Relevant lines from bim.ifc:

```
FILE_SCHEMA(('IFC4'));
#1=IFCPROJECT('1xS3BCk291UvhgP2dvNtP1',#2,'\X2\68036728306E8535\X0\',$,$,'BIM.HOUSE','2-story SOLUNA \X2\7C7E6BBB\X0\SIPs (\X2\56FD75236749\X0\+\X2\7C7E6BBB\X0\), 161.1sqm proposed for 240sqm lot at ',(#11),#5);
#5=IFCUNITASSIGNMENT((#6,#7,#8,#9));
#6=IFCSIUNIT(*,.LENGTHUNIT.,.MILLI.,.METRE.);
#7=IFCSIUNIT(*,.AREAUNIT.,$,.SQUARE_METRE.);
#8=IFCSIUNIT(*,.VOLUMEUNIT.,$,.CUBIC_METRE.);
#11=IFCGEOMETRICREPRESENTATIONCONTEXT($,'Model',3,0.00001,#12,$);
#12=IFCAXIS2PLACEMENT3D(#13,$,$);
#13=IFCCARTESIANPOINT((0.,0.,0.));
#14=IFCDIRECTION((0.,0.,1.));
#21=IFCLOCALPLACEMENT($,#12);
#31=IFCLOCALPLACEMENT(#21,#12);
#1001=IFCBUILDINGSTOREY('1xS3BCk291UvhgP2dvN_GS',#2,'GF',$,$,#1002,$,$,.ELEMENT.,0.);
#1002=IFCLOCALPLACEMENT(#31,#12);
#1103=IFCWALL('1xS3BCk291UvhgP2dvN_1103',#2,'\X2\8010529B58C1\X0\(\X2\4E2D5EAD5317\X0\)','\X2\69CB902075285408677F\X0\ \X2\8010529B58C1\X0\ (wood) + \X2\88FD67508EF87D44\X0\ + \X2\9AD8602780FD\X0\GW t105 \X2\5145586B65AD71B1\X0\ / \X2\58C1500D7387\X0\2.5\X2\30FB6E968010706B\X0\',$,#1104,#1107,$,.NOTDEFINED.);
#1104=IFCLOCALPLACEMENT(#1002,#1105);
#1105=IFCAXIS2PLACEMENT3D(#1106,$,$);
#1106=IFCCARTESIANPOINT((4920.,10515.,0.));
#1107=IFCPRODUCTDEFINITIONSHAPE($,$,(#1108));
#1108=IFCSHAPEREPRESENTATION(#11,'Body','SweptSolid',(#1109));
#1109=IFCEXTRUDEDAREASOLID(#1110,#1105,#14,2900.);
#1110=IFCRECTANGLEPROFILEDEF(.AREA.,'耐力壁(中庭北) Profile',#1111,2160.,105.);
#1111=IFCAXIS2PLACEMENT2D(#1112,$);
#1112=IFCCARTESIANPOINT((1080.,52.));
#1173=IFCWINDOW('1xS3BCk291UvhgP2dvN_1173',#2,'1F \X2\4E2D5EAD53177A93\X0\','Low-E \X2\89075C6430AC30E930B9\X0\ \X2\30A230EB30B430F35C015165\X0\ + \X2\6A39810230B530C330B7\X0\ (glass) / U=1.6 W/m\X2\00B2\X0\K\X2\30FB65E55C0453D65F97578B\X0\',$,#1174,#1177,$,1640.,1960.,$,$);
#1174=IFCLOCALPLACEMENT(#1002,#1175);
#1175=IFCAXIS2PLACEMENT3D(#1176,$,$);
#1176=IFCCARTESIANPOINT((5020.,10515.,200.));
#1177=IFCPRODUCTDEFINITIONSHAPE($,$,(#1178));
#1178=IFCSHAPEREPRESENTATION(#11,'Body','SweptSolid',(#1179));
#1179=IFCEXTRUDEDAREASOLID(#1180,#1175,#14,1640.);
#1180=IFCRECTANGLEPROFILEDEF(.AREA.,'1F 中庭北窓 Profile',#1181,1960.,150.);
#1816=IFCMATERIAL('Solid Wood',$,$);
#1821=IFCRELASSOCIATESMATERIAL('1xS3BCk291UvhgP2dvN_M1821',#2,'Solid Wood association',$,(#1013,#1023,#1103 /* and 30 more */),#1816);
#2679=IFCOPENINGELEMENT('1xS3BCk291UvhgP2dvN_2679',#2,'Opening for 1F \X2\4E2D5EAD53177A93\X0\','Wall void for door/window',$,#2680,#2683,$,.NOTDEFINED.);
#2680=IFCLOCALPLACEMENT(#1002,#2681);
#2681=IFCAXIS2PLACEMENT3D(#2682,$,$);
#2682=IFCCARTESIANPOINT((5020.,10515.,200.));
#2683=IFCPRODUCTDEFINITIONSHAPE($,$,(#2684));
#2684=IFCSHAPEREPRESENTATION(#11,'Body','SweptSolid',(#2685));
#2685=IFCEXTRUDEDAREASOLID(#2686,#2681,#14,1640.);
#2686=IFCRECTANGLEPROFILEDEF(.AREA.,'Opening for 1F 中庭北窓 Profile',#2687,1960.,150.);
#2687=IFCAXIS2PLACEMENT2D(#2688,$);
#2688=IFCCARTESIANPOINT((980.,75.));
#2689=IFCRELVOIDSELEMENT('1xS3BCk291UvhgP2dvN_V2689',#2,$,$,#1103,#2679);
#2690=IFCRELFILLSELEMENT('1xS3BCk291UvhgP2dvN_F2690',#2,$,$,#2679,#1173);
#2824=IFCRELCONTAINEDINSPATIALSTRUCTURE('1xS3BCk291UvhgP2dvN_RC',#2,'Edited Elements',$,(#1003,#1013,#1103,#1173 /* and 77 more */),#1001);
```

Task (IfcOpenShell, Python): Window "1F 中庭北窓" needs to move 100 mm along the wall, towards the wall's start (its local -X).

```python
import ifcopenshell
import ifcopenshell.api.geometry
import ifcopenshell.util.placement
import ifcopenshell.util.unit

model = ifcopenshell.open("bim.ifc")
unit_scale = ifcopenshell.util.unit.calculate_unit_scale(model)

window = model.by_id(1173)
opening = window.FillsVoids[0].RelatingOpeningElement
wall = opening.VoidsElements[0].RelatingBuildingElement

wall_matrix = ifcopenshell.util.placement.get_local_placement(wall.ObjectPlacement)
shift = wall_matrix[:3, 0] * -0.1 / unit_scale
before = ifcopenshell.util.placement.get_local_placement(window.ObjectPlacement)[:3, 3].copy()

# The window is not placed relative to its opening, so move both.
for product in (opening, window):
    matrix = ifcopenshell.util.placement.get_local_placement(product.ObjectPlacement)
    matrix[:3, 3] += shift
    ifcopenshell.api.geometry.edit_object_placement(model, product=product, matrix=matrix, is_si=False)

after = ifcopenshell.util.placement.get_local_placement(window.ObjectPlacement)[:3, 3]
print("window moved by", (after - before).round(3) + 0.0)

model.write("bim_rev.ifc")
```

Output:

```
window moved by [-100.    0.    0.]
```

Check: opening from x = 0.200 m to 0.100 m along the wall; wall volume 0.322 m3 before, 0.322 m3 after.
